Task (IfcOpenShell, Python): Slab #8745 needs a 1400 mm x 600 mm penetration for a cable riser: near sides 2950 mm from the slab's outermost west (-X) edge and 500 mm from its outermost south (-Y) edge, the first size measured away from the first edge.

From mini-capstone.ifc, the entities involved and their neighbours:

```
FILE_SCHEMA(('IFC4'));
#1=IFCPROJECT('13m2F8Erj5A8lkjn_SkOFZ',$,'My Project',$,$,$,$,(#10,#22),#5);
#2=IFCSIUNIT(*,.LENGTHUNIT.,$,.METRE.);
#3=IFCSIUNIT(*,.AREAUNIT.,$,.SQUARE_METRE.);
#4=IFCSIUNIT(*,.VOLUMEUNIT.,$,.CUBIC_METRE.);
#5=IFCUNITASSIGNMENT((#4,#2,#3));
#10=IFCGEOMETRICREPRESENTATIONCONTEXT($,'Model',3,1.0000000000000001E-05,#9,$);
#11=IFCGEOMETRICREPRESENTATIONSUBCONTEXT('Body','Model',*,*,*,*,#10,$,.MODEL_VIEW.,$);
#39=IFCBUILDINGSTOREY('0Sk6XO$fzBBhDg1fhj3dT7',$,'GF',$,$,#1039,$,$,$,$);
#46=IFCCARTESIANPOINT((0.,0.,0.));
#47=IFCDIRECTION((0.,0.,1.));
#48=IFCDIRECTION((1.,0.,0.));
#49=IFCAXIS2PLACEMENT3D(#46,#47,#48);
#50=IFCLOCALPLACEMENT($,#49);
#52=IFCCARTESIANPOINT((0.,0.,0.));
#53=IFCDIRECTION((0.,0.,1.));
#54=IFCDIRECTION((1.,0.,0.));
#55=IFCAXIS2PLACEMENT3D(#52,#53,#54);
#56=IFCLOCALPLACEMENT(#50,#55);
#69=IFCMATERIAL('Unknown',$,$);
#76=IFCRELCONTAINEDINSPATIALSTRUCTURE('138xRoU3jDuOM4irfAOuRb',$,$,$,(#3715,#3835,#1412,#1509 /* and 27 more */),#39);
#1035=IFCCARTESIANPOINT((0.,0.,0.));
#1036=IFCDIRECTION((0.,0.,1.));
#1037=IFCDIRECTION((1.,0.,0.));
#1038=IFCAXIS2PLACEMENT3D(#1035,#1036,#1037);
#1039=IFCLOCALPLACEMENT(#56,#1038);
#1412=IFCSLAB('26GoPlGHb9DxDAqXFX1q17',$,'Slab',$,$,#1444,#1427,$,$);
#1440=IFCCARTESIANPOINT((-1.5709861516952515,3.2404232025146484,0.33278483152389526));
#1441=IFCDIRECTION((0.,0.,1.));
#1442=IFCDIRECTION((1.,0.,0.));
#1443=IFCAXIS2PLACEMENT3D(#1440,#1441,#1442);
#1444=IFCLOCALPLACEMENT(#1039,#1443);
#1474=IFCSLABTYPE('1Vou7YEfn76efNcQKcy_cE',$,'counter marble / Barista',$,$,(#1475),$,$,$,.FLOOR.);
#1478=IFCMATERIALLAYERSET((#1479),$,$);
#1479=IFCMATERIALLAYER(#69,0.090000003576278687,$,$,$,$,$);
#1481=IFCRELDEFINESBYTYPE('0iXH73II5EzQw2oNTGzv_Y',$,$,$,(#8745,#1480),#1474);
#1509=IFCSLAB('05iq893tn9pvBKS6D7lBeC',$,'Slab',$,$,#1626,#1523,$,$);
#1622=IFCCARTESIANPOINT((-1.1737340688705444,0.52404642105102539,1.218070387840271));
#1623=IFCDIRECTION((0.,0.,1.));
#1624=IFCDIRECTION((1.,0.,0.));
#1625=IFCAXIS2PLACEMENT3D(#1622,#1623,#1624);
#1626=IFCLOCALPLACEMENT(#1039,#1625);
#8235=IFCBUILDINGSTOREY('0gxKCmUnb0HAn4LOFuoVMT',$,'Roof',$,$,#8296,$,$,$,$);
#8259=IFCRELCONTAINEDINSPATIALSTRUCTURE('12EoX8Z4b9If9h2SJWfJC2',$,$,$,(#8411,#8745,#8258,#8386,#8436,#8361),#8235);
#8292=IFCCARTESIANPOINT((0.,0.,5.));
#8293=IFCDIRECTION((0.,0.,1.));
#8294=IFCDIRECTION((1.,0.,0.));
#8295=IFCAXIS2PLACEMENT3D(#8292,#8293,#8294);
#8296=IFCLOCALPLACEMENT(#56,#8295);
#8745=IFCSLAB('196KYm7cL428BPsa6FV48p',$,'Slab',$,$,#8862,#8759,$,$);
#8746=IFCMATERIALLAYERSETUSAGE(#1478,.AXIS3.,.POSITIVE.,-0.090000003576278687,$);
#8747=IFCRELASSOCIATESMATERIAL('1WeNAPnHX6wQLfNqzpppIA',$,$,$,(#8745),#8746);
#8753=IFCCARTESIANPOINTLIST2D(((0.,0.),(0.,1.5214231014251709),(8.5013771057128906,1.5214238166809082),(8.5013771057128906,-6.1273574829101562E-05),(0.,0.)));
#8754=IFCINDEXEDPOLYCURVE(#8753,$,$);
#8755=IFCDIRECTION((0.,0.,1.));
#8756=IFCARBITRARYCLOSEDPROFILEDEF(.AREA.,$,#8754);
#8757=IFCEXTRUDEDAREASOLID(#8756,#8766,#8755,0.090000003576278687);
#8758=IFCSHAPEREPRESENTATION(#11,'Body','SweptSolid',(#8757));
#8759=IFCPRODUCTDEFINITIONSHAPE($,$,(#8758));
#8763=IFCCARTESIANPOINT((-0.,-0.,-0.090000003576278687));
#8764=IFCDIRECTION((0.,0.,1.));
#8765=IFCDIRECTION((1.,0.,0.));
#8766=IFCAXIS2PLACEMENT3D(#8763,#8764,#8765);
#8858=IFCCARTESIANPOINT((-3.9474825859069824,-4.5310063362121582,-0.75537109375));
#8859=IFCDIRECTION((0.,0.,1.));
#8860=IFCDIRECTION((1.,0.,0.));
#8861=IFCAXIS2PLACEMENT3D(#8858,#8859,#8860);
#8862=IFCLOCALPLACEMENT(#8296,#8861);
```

```python
import numpy as np
import ifcopenshell
import ifcopenshell.api.feature
import ifcopenshell.api.geometry
import ifcopenshell.api.root
import ifcopenshell.geom
import ifcopenshell.util.placement
import ifcopenshell.util.representation
import ifcopenshell.util.shape
import ifcopenshell.util.unit

model = ifcopenshell.open("mini-capstone.ifc")
unit_scale = ifcopenshell.util.unit.calculate_unit_scale(model)
settings = ifcopenshell.geom.settings()


def volume(element):
    """Net volume in cubic metres, openings subtracted."""
    shape = ifcopenshell.geom.create_shape(settings, element)
    return ifcopenshell.util.shape.get_volume(shape.geometry)


slab = model.by_guid("196KYm7cL428BPsa6FV48p")
before = volume(slab)

# Extent in the slab's own axes, in metres. The edges named are its -X and -Y sides.
slab_shape = ifcopenshell.geom.create_shape(settings, slab)
vertices = ifcopenshell.util.shape.get_vertices(slab_shape.geometry)
x_min, y_min, bottom = vertices.min(axis=0)
top = vertices[:, 2].max()

opening = ifcopenshell.api.root.create_entity(model, ifc_class="IfcOpeningElement", name="Cable riser opening", predefined_type="OPENING")
context = ifcopenshell.util.representation.get_context(model, "Model", "Body", "MODEL_VIEW")
width, depth = 1.4, 0.6
outline = [(0.0, 0.0), (width, 0.0), (width, depth), (0.0, depth), (0.0, 0.0)]
# Overshoot both faces by 50 mm so the cut is clean.
shape = ifcopenshell.api.geometry.add_slab_representation(
    model, context=context, depth=top - bottom + 0.1, polyline=outline
)
ifcopenshell.api.geometry.assign_representation(model, product=opening, representation=shape)

matrix = ifcopenshell.util.placement.get_local_placement(slab.ObjectPlacement)
matrix[:, 3] = matrix @ np.append(np.array([x_min + 2.95, y_min + 0.5, bottom - 0.05]) / unit_scale, 1.0)
ifcopenshell.api.geometry.edit_object_placement(model, product=opening, matrix=matrix, is_si=False)
ifcopenshell.api.feature.add_feature(model, feature=opening, element=slab)

after = volume(slab)

print(f"slab volume {before:.3f} -> {after:.3f} m3")

model.write("mini-capstone_updated.ifc")
```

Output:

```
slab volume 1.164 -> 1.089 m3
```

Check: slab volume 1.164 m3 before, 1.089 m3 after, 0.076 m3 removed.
